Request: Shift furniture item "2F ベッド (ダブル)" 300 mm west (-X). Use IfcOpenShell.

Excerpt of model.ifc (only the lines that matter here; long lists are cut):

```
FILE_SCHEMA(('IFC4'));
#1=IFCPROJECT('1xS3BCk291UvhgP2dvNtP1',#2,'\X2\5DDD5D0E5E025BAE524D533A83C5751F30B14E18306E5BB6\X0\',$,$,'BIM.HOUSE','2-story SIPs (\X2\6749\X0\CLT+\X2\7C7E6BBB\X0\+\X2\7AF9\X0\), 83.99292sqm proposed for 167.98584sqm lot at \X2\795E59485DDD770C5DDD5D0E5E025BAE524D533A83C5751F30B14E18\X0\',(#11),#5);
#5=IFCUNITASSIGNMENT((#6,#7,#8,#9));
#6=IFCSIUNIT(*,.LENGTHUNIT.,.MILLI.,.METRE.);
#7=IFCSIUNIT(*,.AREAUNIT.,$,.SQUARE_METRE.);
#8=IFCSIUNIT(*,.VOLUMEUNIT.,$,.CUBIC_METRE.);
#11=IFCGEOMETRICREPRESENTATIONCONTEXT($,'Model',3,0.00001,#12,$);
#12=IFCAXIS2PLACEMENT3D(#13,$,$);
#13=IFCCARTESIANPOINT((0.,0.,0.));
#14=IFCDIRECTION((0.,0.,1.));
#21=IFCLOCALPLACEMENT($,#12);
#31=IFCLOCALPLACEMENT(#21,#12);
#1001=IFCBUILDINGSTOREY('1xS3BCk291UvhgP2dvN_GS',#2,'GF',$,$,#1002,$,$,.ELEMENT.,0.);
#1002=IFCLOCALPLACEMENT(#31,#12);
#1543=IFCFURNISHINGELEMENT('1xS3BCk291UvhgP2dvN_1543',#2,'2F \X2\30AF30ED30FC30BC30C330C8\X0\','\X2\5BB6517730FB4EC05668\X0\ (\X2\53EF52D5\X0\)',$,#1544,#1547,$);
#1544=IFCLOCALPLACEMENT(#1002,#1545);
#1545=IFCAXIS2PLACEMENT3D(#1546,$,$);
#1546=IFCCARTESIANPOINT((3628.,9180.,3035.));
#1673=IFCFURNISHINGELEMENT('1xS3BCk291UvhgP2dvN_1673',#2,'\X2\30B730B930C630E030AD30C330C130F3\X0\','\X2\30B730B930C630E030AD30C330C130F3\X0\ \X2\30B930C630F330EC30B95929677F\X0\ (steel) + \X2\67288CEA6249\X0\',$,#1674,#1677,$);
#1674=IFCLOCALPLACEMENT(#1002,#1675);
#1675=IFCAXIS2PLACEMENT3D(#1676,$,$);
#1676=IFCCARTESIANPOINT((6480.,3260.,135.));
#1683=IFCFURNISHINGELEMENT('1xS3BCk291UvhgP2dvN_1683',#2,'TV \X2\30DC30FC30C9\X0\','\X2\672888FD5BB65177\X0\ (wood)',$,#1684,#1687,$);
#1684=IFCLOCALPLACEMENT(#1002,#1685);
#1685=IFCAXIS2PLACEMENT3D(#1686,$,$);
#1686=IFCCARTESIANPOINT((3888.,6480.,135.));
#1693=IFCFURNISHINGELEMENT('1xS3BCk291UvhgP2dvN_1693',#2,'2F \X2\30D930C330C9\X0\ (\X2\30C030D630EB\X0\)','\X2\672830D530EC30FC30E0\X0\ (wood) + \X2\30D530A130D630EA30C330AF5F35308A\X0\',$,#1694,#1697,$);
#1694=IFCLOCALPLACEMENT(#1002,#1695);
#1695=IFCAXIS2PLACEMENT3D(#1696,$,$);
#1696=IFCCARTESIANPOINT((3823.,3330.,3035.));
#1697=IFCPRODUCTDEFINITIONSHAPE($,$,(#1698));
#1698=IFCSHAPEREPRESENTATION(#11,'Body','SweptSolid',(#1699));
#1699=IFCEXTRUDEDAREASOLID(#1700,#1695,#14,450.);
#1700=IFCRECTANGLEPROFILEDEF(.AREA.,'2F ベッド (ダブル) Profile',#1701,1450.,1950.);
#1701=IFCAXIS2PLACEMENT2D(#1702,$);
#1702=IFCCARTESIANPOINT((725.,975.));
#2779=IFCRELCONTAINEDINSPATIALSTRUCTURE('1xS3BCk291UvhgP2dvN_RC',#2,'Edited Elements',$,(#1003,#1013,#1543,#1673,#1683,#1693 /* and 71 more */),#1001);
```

```python
import ifcopenshell
import ifcopenshell.api.geometry
import ifcopenshell.util.placement

model = ifcopenshell.open("model.ifc")

item = model.by_guid("1xS3BCk291UvhgP2dvN_1693")
matrix = ifcopenshell.util.placement.get_local_placement(item.ObjectPlacement)
matrix[0, 3] -= 300.0
ifcopenshell.api.geometry.edit_object_placement(model, product=item, matrix=matrix, is_si=False)

print(ifcopenshell.util.placement.get_local_placement(item.ObjectPlacement).round(3) + 0.0)

model.write("model_v2.ifc")
```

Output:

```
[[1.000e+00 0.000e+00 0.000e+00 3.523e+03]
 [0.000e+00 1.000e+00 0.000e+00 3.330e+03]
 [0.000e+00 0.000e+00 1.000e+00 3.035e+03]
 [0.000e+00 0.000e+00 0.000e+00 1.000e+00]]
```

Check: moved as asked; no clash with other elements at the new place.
